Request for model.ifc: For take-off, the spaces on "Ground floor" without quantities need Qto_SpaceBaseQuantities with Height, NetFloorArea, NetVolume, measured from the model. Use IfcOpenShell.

First a look at what the model holds.

```python
import ifcopenshell
import ifcopenshell.util.element
import ifcopenshell.util.unit

model = ifcopenshell.open("model.ifc")
print(model.schema)
for unit_type in ("LENGTHUNIT", "AREAUNIT", "VOLUMEUNIT"):
    print(unit_type, ifcopenshell.util.unit.calculate_unit_scale(model, unit_type))
storey = next(s for s in model.by_type("IfcBuildingStorey") if s.Name == "Ground floor")
spaces = [e for e in ifcopenshell.util.element.get_decomposition(storey) if e.is_a("IfcSpace")]
for e in sorted(spaces, key=lambda e: e.id()):
    print(e.id(), e.is_a(), e.Name, list(ifcopenshell.util.element.get_psets(e, qtos_only=True)), sep=" | ")
```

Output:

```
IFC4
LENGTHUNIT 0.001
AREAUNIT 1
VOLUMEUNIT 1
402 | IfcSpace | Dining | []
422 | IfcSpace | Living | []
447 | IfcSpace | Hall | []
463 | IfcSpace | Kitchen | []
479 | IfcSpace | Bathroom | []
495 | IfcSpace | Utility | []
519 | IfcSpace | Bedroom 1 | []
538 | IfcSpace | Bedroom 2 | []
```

```python
import ifcopenshell
import ifcopenshell.api.pset
import ifcopenshell.geom
import ifcopenshell.util.element
import ifcopenshell.util.shape
import ifcopenshell.util.unit

model = ifcopenshell.open("model.ifc")
unit_scale = ifcopenshell.util.unit.calculate_unit_scale(model)
area_scale = ifcopenshell.util.unit.calculate_unit_scale(model, "AREAUNIT")
volume_scale = ifcopenshell.util.unit.calculate_unit_scale(model, "VOLUMEUNIT")
settings = ifcopenshell.geom.settings()

storey = next(s for s in model.by_type("IfcBuildingStorey") if s.Name == "Ground floor")
spaces = [e for e in ifcopenshell.util.element.get_decomposition(storey) if e.is_a("IfcSpace")]

for e in sorted(spaces, key=lambda e: e.id()):
    if ifcopenshell.util.element.get_psets(e, qtos_only=True, should_inherit=False):
        continue
    # Geometry comes back in metres, in the element's own axes.
    shape = ifcopenshell.geom.create_shape(settings, e)
    values = {
        "Height": ifcopenshell.util.shape.get_z(shape.geometry) / unit_scale,
        "NetFloorArea": ifcopenshell.util.shape.get_footprint_area(shape.geometry) / area_scale,
        "NetVolume": ifcopenshell.util.shape.get_volume(shape.geometry) / volume_scale,
    }
    qto = ifcopenshell.api.pset.add_qto(model, product=e, name="Qto_SpaceBaseQuantities")
    ifcopenshell.api.pset.edit_qto(model, qto=qto, properties=values)
    print(e.id(), {k: round(v, 3) for k, v in values.items()})

model.write("model-out.ifc")
```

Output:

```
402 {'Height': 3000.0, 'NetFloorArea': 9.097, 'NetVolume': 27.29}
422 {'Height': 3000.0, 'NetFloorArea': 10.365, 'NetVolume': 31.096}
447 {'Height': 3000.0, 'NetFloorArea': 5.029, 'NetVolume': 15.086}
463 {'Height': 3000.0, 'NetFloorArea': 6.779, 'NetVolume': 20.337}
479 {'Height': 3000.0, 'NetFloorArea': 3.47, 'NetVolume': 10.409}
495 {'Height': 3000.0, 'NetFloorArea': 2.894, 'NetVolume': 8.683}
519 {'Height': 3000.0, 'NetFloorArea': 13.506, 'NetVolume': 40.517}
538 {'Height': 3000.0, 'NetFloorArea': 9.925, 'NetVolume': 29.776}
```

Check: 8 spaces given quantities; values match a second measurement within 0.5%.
